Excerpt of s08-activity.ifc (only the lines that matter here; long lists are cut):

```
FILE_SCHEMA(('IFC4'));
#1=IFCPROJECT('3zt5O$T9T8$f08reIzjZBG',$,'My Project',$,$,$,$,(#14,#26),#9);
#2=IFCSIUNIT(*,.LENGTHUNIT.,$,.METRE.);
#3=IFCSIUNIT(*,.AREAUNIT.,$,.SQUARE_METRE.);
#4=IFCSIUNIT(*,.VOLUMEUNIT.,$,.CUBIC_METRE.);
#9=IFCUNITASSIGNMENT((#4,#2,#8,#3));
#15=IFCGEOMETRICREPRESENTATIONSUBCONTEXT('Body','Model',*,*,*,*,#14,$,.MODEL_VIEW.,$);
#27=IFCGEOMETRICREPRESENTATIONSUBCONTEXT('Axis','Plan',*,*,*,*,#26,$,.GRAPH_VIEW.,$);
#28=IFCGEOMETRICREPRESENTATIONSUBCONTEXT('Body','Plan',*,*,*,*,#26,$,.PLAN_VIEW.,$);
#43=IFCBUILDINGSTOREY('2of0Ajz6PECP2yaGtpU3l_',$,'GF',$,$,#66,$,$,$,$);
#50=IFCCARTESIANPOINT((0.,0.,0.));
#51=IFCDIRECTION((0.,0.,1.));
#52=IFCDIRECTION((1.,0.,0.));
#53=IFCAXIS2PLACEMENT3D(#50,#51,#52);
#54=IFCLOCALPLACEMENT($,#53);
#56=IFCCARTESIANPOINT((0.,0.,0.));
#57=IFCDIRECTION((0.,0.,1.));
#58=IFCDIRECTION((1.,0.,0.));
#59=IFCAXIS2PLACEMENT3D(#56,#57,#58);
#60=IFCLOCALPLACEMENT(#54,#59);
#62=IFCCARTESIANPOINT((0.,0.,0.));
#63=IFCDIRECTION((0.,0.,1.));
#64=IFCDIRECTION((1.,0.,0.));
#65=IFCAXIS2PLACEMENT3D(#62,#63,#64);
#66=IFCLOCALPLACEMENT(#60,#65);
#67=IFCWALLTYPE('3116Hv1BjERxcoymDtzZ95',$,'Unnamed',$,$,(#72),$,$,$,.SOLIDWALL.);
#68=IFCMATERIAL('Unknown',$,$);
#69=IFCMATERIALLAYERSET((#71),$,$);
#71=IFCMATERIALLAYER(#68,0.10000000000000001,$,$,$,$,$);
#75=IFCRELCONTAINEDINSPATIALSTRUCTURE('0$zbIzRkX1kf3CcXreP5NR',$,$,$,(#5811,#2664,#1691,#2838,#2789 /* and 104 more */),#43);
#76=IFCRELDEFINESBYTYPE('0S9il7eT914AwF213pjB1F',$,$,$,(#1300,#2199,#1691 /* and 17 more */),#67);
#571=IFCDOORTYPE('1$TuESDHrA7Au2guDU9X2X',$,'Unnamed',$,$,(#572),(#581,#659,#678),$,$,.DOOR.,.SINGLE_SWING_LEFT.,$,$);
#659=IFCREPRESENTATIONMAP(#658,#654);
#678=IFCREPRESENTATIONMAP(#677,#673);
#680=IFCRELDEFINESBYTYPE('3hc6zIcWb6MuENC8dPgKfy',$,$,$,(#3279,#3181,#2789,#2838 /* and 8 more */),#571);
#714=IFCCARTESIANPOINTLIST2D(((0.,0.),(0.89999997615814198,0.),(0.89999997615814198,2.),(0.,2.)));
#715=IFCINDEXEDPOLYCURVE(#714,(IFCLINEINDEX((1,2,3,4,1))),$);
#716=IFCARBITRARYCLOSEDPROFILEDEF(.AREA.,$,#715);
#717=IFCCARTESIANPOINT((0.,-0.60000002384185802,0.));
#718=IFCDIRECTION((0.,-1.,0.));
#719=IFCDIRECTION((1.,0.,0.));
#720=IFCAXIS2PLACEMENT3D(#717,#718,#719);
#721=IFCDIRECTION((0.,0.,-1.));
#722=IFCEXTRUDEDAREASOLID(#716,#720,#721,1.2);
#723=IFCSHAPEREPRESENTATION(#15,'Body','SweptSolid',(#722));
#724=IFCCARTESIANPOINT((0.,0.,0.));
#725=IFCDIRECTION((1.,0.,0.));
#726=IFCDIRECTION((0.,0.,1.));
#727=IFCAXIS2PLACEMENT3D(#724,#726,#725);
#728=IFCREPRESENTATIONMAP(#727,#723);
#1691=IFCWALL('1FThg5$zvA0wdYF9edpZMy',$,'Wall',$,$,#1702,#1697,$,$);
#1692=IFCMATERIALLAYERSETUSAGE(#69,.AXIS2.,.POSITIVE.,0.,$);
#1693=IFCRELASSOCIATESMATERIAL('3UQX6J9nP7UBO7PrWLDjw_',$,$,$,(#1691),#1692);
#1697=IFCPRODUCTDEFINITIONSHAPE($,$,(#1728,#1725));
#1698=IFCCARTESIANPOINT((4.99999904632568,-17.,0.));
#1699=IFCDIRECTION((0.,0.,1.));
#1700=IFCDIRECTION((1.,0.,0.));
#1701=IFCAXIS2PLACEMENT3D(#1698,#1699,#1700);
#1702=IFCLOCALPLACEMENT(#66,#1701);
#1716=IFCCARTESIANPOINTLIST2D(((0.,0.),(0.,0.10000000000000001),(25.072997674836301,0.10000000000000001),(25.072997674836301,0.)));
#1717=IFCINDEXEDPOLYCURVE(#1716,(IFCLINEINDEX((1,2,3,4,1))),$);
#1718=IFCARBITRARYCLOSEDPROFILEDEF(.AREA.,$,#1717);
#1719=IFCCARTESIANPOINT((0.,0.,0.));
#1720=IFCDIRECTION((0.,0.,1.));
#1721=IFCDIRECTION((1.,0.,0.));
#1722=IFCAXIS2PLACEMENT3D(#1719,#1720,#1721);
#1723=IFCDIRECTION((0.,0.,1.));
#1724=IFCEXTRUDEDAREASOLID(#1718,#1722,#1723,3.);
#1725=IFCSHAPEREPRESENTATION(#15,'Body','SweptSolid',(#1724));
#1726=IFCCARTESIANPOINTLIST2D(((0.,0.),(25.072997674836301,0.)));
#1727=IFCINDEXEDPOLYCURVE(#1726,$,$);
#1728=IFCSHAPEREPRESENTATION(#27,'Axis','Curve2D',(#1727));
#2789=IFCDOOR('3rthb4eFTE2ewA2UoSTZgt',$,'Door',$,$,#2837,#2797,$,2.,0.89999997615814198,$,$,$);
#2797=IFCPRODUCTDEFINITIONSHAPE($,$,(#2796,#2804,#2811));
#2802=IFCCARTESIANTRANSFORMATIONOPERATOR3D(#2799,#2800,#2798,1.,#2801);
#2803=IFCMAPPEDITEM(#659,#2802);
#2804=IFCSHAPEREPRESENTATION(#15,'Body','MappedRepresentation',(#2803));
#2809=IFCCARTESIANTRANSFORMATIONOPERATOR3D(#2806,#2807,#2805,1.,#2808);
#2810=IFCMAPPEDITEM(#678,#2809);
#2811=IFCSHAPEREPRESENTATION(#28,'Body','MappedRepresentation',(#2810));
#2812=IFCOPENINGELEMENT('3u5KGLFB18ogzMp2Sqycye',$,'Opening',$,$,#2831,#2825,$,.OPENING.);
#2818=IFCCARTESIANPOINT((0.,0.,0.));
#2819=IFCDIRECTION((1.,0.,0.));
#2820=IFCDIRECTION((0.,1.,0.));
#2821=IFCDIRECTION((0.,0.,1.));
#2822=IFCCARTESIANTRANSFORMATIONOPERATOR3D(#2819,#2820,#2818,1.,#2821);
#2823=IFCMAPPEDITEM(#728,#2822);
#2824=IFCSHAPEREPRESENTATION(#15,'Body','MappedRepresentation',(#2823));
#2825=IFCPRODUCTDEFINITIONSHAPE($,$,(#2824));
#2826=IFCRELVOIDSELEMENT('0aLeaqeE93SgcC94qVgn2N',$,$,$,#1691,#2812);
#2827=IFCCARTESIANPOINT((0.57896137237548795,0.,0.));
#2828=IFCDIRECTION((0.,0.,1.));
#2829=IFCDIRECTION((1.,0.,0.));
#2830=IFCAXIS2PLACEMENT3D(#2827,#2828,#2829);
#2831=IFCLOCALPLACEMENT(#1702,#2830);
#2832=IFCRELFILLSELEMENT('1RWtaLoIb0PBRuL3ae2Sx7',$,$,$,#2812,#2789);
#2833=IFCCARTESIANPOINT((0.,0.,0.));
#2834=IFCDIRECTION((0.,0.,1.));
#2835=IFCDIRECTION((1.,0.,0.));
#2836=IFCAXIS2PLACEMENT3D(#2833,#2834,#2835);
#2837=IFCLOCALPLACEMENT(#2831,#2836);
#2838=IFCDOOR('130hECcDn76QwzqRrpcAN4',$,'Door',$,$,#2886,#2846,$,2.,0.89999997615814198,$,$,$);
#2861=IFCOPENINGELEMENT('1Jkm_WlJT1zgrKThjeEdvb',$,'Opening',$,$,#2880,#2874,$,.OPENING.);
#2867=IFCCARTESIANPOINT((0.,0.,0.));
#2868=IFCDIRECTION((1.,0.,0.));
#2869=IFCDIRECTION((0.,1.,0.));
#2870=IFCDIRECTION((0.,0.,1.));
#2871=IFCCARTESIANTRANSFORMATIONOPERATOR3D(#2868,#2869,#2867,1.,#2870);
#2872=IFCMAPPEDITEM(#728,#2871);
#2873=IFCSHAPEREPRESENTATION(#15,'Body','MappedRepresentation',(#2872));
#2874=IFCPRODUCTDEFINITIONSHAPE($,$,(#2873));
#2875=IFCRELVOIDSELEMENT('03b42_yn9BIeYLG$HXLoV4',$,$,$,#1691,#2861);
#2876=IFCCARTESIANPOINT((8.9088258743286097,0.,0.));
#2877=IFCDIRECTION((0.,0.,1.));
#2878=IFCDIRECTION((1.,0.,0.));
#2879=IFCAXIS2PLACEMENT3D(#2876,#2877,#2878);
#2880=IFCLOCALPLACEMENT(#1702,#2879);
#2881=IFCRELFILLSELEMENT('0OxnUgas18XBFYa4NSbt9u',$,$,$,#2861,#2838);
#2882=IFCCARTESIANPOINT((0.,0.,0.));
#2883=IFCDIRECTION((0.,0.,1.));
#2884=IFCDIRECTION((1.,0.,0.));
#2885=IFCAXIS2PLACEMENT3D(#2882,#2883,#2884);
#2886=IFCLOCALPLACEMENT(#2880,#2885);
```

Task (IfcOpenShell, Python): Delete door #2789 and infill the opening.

```python
import ifcopenshell
import ifcopenshell.api.feature
import ifcopenshell.api.root
import ifcopenshell.geom
import ifcopenshell.util.shape

model = ifcopenshell.open("s08-activity.ifc")
settings = ifcopenshell.geom.settings()


def volume(element):
    """Net volume in cubic metres, openings subtracted."""
    shape = ifcopenshell.geom.create_shape(settings, element)
    return ifcopenshell.util.shape.get_volume(shape.geometry)


door = model.by_guid("3rthb4eFTE2ewA2UoSTZgt")
opening = door.FillsVoids[0].RelatingOpeningElement
wall = opening.VoidsElements[0].RelatingBuildingElement
before = volume(wall)

ifcopenshell.api.root.remove_product(model, product=door)
ifcopenshell.api.feature.remove_feature(model, feature=opening)

after = volume(wall)

print(f"wall volume {before:.3f} -> {after:.3f} m3")

model.write("s08-activity_rev.ifc")
```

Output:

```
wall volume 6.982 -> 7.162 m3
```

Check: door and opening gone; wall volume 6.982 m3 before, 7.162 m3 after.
